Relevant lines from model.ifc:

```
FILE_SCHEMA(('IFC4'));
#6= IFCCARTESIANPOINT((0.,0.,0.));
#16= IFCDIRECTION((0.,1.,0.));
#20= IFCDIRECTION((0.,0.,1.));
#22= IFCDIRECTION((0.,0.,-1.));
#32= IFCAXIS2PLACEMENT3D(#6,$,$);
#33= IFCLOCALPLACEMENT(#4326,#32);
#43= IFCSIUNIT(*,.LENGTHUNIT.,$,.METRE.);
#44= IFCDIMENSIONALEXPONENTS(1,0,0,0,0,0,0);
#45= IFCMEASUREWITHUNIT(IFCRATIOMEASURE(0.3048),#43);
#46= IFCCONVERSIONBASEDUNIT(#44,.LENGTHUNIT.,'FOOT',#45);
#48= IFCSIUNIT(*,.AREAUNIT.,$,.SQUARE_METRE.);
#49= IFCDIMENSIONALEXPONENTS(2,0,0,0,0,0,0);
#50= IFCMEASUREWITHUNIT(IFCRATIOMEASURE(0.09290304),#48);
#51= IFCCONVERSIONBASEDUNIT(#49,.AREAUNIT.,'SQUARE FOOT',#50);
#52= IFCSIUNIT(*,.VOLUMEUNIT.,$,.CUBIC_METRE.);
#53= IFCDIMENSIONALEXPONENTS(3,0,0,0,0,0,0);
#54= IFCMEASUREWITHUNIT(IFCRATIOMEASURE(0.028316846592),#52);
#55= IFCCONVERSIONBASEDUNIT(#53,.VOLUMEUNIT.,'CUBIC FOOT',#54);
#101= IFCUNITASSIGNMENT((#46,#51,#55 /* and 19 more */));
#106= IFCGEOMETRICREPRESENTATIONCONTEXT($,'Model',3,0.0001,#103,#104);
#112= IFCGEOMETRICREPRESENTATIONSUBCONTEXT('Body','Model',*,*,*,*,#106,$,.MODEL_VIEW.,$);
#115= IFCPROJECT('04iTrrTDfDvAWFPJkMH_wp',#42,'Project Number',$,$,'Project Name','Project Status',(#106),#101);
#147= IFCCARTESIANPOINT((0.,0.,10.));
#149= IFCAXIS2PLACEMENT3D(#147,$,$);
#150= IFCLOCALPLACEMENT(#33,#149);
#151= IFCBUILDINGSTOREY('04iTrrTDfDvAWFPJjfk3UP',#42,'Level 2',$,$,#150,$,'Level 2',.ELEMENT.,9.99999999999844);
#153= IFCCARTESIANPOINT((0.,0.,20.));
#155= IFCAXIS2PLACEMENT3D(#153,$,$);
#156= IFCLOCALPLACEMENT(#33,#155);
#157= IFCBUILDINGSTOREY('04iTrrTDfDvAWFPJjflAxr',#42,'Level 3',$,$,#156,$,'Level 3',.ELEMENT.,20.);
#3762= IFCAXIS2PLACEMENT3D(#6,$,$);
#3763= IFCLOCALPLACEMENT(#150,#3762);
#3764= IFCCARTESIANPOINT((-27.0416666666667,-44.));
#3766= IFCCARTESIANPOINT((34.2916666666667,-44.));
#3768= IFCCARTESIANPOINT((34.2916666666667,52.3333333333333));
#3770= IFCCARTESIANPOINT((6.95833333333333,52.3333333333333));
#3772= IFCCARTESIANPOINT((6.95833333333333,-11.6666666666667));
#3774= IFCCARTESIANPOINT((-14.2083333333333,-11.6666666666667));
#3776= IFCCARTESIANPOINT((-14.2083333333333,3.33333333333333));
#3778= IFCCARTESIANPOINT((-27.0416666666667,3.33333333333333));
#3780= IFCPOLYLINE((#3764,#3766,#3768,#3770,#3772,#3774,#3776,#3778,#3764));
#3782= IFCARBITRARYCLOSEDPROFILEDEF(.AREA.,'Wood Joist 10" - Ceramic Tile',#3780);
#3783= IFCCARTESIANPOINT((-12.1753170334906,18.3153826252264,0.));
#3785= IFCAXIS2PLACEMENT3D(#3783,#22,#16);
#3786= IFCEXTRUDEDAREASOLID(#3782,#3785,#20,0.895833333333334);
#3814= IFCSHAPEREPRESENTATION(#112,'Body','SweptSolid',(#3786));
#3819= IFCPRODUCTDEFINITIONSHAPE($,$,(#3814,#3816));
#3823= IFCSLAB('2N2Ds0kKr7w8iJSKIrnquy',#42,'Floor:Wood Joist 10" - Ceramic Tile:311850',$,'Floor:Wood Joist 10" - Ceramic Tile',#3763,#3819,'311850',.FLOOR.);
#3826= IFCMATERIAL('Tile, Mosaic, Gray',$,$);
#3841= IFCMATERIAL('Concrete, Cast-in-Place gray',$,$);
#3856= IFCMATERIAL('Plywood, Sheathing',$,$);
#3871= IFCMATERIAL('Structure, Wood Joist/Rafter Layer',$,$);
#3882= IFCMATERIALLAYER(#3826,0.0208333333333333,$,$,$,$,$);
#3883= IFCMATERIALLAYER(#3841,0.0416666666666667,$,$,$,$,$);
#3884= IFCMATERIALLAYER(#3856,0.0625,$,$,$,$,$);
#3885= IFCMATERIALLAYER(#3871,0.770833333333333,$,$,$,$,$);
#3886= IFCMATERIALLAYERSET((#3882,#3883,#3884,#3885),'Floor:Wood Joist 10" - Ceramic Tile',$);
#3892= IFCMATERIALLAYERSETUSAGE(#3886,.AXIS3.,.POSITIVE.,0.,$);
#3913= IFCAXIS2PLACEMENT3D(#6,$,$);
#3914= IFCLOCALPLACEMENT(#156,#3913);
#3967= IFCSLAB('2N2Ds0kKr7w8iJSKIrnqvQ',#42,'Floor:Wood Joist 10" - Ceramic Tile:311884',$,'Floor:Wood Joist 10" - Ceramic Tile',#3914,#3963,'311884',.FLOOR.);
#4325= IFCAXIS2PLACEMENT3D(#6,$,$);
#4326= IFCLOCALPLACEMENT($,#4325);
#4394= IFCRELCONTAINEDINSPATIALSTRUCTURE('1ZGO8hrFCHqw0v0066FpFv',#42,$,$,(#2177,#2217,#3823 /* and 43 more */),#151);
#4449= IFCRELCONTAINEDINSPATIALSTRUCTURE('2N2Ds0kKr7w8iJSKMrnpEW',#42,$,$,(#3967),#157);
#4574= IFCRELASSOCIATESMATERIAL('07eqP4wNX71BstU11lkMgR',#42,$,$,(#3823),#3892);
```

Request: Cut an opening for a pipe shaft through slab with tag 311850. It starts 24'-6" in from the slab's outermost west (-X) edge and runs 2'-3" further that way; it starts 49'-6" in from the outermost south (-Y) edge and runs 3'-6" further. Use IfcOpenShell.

```python
import numpy as np
import ifcopenshell
import ifcopenshell.api.feature
import ifcopenshell.api.geometry
import ifcopenshell.api.root
import ifcopenshell.geom
import ifcopenshell.util.placement
import ifcopenshell.util.representation
import ifcopenshell.util.shape
import ifcopenshell.util.unit

model = ifcopenshell.open("model.ifc")
unit_scale = ifcopenshell.util.unit.calculate_unit_scale(model)
settings = ifcopenshell.geom.settings()


def volume(element):
    """Net volume in cubic metres, openings subtracted."""
    shape = ifcopenshell.geom.create_shape(settings, element)
    return ifcopenshell.util.shape.get_volume(shape.geometry)


slab = model.by_id(3823)
before = volume(slab)

# Extent in the slab's own axes, in metres. The edges named are its -X and -Y sides.
slab_shape = ifcopenshell.geom.create_shape(settings, slab)
vertices = ifcopenshell.util.shape.get_vertices(slab_shape.geometry)
x_min, y_min, bottom = vertices.min(axis=0)
top = vertices[:, 2].max()

opening = ifcopenshell.api.root.create_entity(model, ifc_class="IfcOpeningElement", name="Pipe shaft opening", predefined_type="OPENING")
context = ifcopenshell.util.representation.get_context(model, "Model", "Body", "MODEL_VIEW")
width, depth = 0.6858, 1.0668
outline = [(0.0, 0.0), (width, 0.0), (width, depth), (0.0, depth), (0.0, 0.0)]
# Overshoot both faces by 50 mm so the cut is clean.
shape = ifcopenshell.api.geometry.add_slab_representation(
    model, context=context, depth=top - bottom + 0.1, polyline=outline
)
ifcopenshell.api.geometry.assign_representation(model, product=opening, representation=shape)

matrix = ifcopenshell.util.placement.get_local_placement(slab.ObjectPlacement)
matrix[:, 3] = matrix @ np.append(np.array([x_min + 7.4676, y_min + 15.0876, bottom - 0.05]) / unit_scale, 1.0)
ifcopenshell.api.geometry.edit_object_placement(model, product=opening, matrix=matrix, is_si=False)
ifcopenshell.api.feature.add_feature(model, feature=opening, element=slab)

after = volume(slab)

print(f"slab volume {before:.3f} -> {after:.3f} m3")

model.write("model_rev.ifc")
```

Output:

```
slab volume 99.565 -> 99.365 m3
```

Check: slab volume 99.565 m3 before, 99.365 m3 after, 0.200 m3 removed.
